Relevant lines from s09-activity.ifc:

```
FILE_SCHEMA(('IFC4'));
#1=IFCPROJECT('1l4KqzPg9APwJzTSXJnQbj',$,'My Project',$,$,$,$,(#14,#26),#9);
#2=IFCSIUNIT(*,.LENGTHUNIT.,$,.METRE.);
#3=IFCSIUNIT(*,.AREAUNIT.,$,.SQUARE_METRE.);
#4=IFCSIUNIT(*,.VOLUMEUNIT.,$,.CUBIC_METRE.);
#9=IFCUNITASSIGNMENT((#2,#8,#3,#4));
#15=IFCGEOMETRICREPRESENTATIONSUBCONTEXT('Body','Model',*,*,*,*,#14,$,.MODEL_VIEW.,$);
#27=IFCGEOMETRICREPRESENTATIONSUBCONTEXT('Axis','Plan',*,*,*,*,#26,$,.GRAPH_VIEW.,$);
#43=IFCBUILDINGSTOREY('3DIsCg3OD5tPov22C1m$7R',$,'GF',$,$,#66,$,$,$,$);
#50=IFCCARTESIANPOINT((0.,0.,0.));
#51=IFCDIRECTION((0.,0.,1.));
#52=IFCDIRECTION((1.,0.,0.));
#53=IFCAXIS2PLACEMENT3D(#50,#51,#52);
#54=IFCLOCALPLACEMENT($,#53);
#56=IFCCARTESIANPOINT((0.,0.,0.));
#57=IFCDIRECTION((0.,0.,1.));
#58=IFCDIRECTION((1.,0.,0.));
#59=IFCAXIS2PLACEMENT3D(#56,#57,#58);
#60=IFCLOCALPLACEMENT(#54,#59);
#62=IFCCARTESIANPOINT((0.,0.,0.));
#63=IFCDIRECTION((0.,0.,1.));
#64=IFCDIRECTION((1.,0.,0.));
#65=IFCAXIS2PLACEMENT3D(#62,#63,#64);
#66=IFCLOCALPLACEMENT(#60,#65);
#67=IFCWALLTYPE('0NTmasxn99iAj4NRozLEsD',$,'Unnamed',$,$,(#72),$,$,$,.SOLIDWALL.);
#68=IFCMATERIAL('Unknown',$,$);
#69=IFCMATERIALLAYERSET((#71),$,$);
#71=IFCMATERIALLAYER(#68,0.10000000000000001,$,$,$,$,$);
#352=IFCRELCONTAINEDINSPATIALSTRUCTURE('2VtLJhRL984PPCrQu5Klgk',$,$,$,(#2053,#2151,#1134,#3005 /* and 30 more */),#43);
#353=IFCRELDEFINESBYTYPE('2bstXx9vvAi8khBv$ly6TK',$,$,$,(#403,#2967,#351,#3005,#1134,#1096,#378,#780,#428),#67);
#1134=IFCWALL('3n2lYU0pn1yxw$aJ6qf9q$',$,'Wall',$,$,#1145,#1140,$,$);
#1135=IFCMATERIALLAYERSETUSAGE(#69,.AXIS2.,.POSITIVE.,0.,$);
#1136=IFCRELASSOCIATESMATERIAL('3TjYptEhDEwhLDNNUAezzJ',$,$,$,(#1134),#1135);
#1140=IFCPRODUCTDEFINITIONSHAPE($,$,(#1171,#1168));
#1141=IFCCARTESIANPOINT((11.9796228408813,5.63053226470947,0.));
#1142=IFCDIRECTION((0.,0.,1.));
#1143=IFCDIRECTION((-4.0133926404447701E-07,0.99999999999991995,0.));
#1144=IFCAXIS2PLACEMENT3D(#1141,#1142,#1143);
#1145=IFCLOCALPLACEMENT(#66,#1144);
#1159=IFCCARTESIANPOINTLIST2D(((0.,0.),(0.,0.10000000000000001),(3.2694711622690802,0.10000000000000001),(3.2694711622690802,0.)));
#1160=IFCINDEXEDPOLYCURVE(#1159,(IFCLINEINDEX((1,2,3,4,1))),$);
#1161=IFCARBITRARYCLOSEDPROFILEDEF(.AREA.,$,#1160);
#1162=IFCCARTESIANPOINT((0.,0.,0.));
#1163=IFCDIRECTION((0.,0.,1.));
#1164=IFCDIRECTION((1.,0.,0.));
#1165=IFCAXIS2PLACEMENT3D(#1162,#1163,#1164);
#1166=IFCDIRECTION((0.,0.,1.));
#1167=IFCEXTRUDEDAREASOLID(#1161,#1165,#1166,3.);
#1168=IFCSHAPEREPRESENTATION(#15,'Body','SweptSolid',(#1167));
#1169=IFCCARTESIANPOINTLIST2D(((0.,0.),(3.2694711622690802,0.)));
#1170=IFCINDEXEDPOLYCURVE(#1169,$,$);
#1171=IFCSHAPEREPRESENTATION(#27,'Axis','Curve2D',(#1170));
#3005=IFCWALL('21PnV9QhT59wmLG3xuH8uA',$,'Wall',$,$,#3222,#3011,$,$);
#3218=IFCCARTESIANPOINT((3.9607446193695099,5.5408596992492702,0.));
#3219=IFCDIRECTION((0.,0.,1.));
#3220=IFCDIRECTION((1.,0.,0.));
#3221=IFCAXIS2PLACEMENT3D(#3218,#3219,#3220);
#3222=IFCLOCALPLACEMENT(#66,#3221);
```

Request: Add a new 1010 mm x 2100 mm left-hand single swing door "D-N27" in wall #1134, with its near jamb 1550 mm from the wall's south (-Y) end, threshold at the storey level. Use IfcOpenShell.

```python
import numpy as np
import ifcopenshell
import ifcopenshell.api.feature
import ifcopenshell.api.geometry
import ifcopenshell.api.root
import ifcopenshell.api.spatial
import ifcopenshell.geom
import ifcopenshell.util.element
import ifcopenshell.util.placement
import ifcopenshell.util.representation
import ifcopenshell.util.shape
import ifcopenshell.util.unit

model = ifcopenshell.open("s09-activity.ifc")
unit_scale = ifcopenshell.util.unit.calculate_unit_scale(model)
settings = ifcopenshell.geom.settings()


def volume(element):
    """Net volume in cubic metres, openings subtracted."""
    shape = ifcopenshell.geom.create_shape(settings, element)
    return ifcopenshell.util.shape.get_volume(shape.geometry)


wall = model.by_guid("3n2lYU0pn1yxw$aJ6qf9q$")
storey = ifcopenshell.util.element.get_container(wall, ifc_class="IfcBuildingStorey")
context = ifcopenshell.util.representation.get_context(model, "Model", "Body", "MODEL_VIEW")
before = volume(wall)

width, height, from_end, sill = 1.01, 2.1, 1.55, 0.0  # metres

# The wall runs along its own X axis, and the end named is its -X end.
wall_shape = ifcopenshell.geom.create_shape(settings, wall)
x, y, z = ifcopenshell.util.shape.get_vertices(wall_shape.geometry).T
start = x.min() + from_end
face, thickness = float(y.min()), float(y.max() - y.min())
wall_matrix = ifcopenshell.util.placement.get_local_placement(wall.ObjectPlacement)
level = ifcopenshell.util.placement.get_local_placement(storey.ObjectPlacement)[2, 3]


def in_wall(x, y):
    """Placement at x, y metres in the wall's axes, at sill height."""
    matrix = wall_matrix.copy()
    matrix[:, 3] = wall_matrix @ np.array([x / unit_scale, y / unit_scale, 0.0, 1.0])
    matrix[2, 3] = level + sill / unit_scale
    return matrix


# Opening: a box that overshoots both wall faces by 50 mm.
opening = ifcopenshell.api.root.create_entity(model, ifc_class="IfcOpeningElement", predefined_type="OPENING")
box = ifcopenshell.api.geometry.add_wall_representation(
    model, context=context, length=width, height=height, thickness=thickness + 0.1
)
ifcopenshell.api.geometry.assign_representation(model, product=opening, representation=box)
ifcopenshell.api.geometry.edit_object_placement(model, product=opening, matrix=in_wall(start, face - 0.05), is_si=False)
ifcopenshell.api.feature.add_feature(model, feature=opening, element=wall)

door = ifcopenshell.api.root.create_entity(model, ifc_class="IfcDoor", name="D-N27", predefined_type="DOOR")
door.OverallWidth, door.OverallHeight = width / unit_scale, height / unit_scale
door.OperationType = "SINGLE_SWING_LEFT"
body = ifcopenshell.api.geometry.add_door_representation(
    model,
    context=context,
    overall_width=door.OverallWidth,
    overall_height=door.OverallHeight,
    operation_type="SINGLE_SWING_LEFT",
    lining_properties={"LiningDepth": thickness / unit_scale, "ThresholdDepth": thickness / unit_scale},
)
ifcopenshell.api.geometry.assign_representation(model, product=door, representation=body)
ifcopenshell.api.spatial.assign_container(model, products=[door], relating_structure=storey)
ifcopenshell.api.feature.add_filling(model, opening=opening, element=door)

# The lining spans the wall, so the door starts at the wall face.
ifcopenshell.api.geometry.edit_object_placement(model, product=door, matrix=in_wall(start, face), is_si=False)

after = volume(wall)

print(f"wall volume {before:.3f} -> {after:.3f} m3")

model.write("s09-activity_v2.ifc")
```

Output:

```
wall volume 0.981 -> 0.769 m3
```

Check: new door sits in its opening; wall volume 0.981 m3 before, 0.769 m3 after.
